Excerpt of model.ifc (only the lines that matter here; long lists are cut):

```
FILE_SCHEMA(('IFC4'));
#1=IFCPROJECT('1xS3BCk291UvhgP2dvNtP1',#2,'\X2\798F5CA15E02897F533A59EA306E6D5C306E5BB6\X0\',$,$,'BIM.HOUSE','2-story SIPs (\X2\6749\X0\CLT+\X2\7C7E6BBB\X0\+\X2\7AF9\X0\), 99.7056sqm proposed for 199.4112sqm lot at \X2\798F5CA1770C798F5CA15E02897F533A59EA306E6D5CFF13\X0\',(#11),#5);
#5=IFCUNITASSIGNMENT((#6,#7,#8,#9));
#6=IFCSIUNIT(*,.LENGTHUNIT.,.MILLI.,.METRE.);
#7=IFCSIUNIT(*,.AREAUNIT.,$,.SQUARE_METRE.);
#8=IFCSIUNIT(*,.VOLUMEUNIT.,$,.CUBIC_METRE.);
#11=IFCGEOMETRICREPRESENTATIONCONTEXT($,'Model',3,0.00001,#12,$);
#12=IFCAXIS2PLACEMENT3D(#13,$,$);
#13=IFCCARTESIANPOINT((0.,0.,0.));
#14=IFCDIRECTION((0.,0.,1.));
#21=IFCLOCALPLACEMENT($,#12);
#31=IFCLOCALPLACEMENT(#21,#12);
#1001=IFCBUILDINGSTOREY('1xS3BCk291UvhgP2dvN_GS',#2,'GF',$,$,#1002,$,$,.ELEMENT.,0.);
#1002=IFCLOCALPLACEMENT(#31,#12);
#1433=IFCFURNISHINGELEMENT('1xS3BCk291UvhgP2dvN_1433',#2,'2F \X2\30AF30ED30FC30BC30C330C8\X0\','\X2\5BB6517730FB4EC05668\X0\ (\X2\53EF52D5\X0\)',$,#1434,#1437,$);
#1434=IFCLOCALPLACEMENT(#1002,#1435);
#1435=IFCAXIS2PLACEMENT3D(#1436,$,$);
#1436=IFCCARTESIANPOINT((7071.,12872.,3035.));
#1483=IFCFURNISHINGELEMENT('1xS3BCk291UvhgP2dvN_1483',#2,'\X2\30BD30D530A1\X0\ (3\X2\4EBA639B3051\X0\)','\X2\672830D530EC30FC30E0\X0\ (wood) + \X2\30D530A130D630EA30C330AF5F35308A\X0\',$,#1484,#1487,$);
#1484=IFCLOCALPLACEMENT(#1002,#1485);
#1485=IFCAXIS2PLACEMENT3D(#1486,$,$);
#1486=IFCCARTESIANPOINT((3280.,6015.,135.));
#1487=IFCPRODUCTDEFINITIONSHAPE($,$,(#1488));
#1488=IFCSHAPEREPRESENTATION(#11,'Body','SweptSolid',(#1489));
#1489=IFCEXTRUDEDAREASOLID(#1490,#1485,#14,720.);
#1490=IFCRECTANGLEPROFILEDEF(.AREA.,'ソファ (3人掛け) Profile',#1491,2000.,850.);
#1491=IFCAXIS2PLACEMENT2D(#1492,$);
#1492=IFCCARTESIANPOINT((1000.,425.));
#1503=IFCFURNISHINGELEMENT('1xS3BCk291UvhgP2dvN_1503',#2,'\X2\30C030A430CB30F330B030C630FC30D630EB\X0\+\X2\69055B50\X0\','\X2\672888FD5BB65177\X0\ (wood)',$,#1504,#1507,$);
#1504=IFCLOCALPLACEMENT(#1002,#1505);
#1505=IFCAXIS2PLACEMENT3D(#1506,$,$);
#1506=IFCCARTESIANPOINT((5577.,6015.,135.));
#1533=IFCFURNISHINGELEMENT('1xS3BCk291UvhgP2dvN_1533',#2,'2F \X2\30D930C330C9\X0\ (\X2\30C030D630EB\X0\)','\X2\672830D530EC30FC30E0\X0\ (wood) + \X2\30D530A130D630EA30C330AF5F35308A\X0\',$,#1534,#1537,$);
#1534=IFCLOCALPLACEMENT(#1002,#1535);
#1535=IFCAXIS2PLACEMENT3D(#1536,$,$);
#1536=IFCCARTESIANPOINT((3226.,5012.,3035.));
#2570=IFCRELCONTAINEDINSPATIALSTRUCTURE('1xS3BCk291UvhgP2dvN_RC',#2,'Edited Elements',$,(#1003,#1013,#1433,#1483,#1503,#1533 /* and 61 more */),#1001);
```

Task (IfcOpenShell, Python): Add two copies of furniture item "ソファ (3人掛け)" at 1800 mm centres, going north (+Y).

```python
import numpy as np
import ifcopenshell
import ifcopenshell.api.geometry
import ifcopenshell.api.root
import ifcopenshell.util.element
import ifcopenshell.util.placement

model = ifcopenshell.open("model.ifc")


def reuse_history(source, copy):
    """copy_class also copies each property set's owner history, people and application; keep the originals."""
    for rel in copy.IsDefinedBy:
        if rel.is_a("IfcRelDefinesByProperties") and (history := rel.RelatingPropertyDefinition.OwnerHistory):
            rel.RelatingPropertyDefinition.OwnerHistory = source.OwnerHistory
            ifcopenshell.util.element.remove_deep2(model, history)


source = model.by_guid("1xS3BCk291UvhgP2dvN_1483")
base = ifcopenshell.util.placement.get_local_placement(source.ObjectPlacement)
step = np.array([0.0, 1.0, 0.0]) * 1800.0

for i in range(1, 3):
    copy = ifcopenshell.api.root.copy_class(model, product=source)
    copy.Representation = ifcopenshell.util.element.copy_deep(
        model, source.Representation, exclude=["IfcGeometricRepresentationContext", "IfcRepresentationMap"]
    )
    reuse_history(source, copy)
    matrix = base.copy()
    matrix[:3, 3] += i * step
    print("added at", matrix[:3, 3].round(3) + 0.0)
    ifcopenshell.api.geometry.edit_object_placement(model, product=copy, matrix=matrix, is_si=False)

model.write("model_edited.ifc")
```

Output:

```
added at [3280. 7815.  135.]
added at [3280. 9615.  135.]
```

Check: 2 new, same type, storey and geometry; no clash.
